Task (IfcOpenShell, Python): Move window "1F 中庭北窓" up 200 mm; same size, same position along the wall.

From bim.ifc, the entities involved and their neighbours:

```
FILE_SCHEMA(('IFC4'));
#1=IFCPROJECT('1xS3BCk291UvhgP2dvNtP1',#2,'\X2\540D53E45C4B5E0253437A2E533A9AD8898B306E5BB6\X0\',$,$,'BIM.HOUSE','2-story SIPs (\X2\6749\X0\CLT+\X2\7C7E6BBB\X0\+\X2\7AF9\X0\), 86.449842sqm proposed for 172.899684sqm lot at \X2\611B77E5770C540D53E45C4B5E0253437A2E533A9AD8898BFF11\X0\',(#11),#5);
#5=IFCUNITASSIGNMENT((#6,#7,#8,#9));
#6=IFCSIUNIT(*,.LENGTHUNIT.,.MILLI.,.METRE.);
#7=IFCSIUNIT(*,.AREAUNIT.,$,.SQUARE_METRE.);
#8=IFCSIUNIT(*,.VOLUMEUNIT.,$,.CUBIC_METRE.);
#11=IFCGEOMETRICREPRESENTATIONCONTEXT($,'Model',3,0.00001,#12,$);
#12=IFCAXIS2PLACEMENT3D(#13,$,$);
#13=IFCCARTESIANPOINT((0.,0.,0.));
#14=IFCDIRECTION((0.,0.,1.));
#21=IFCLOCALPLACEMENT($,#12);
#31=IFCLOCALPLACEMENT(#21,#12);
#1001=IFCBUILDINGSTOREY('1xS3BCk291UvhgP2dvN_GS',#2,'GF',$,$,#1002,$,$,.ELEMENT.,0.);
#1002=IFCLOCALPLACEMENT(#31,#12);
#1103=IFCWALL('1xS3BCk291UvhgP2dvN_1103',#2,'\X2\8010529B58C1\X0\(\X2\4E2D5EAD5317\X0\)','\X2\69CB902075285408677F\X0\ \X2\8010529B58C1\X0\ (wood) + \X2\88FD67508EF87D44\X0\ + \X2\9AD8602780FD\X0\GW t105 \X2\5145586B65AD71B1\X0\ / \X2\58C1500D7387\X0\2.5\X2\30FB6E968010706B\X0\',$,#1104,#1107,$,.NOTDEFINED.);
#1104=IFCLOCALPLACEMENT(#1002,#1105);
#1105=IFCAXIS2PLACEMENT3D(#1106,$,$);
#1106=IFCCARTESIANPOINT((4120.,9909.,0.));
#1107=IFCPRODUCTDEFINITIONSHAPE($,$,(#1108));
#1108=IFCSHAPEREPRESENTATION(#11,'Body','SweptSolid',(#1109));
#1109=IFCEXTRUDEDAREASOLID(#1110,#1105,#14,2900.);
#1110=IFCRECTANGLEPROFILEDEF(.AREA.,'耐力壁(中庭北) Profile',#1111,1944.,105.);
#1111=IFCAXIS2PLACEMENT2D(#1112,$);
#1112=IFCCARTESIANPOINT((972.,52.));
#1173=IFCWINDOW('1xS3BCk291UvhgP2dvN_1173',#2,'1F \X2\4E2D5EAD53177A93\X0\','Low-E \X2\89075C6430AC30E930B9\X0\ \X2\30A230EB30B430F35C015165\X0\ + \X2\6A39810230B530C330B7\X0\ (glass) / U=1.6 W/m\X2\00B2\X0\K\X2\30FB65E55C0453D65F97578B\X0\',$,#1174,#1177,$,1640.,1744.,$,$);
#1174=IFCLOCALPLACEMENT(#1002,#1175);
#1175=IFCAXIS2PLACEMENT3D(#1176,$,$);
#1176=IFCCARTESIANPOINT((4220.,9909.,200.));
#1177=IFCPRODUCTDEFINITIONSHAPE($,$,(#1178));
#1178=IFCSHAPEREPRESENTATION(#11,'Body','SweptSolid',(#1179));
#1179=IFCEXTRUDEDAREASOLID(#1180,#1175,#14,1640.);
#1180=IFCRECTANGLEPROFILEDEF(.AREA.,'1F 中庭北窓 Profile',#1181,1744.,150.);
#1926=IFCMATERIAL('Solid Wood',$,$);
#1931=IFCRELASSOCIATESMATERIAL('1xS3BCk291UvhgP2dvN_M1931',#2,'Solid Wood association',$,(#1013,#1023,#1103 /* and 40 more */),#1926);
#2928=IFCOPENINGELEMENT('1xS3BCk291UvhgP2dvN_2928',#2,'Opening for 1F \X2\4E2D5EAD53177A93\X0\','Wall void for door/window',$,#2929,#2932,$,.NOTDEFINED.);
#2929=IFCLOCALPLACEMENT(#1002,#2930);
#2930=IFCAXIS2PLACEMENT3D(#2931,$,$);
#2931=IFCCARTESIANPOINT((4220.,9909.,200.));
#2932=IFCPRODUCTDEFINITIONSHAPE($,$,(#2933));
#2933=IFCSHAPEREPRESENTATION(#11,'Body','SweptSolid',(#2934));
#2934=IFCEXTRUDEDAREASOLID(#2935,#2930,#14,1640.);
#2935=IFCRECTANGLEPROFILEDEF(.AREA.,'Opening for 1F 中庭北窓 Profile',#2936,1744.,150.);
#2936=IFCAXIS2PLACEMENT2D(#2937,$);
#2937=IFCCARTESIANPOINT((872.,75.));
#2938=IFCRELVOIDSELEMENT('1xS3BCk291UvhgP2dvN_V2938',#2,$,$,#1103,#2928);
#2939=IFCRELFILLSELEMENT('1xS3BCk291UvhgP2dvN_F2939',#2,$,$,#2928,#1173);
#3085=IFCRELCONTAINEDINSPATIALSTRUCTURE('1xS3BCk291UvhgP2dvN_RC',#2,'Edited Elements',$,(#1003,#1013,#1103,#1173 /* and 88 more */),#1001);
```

```python
import numpy as np
import ifcopenshell
import ifcopenshell.api.geometry
import ifcopenshell.util.placement
import ifcopenshell.util.unit

model = ifcopenshell.open("bim.ifc")
unit_scale = ifcopenshell.util.unit.calculate_unit_scale(model)

window = model.by_id(1173)
opening = window.FillsVoids[0].RelatingOpeningElement
dz = 200.0

shift = np.array([0.0, 0.0, dz])
# The window is not placed relative to its opening, so move both.
for product in (opening, window):
    matrix = ifcopenshell.util.placement.get_local_placement(product.ObjectPlacement)
    matrix[:3, 3] += shift
    ifcopenshell.api.geometry.edit_object_placement(model, product=product, matrix=matrix, is_si=False)

print(f"moved by {dz * unit_scale:+.3f} m")

model.write("bim-out.ifc")
```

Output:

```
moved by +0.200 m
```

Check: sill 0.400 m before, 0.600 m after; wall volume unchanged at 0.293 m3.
